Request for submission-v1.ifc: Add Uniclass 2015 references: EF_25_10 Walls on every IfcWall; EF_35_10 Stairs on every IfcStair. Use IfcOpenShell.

First a look at what the model holds.

```python
import ifcopenshell

model = ifcopenshell.open("submission-v1.ifc")
print(model.schema)
print("classifications:", [c.Name for c in model.by_type("IfcClassification")])
for ifc_class in ("IfcDoor", "IfcRoof", "IfcStair", "IfcWall", "IfcWindow"):
    print(ifc_class, len(model.by_type(ifc_class)))
```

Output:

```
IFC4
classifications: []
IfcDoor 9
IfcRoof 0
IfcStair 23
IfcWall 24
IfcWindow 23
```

```python
import ifcopenshell
import ifcopenshell.api.classification

model = ifcopenshell.open("submission-v1.ifc")

system = ifcopenshell.api.classification.add_classification(model, classification="Uniclass 2015")

codes = {
    "IfcWall": ("EF_25_10", "Walls"),
    "IfcStair": ("EF_35_10", "Stairs"),
}
for ifc_class, (code, name) in codes.items():
    products = model.by_type(ifc_class)
    ifcopenshell.api.classification.add_reference(
        model, products=products, classification=system, identification=code, name=name
    )
    print(code, len(products))

model.write("submission-v1_edited.ifc")
```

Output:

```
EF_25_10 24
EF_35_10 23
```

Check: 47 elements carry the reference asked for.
